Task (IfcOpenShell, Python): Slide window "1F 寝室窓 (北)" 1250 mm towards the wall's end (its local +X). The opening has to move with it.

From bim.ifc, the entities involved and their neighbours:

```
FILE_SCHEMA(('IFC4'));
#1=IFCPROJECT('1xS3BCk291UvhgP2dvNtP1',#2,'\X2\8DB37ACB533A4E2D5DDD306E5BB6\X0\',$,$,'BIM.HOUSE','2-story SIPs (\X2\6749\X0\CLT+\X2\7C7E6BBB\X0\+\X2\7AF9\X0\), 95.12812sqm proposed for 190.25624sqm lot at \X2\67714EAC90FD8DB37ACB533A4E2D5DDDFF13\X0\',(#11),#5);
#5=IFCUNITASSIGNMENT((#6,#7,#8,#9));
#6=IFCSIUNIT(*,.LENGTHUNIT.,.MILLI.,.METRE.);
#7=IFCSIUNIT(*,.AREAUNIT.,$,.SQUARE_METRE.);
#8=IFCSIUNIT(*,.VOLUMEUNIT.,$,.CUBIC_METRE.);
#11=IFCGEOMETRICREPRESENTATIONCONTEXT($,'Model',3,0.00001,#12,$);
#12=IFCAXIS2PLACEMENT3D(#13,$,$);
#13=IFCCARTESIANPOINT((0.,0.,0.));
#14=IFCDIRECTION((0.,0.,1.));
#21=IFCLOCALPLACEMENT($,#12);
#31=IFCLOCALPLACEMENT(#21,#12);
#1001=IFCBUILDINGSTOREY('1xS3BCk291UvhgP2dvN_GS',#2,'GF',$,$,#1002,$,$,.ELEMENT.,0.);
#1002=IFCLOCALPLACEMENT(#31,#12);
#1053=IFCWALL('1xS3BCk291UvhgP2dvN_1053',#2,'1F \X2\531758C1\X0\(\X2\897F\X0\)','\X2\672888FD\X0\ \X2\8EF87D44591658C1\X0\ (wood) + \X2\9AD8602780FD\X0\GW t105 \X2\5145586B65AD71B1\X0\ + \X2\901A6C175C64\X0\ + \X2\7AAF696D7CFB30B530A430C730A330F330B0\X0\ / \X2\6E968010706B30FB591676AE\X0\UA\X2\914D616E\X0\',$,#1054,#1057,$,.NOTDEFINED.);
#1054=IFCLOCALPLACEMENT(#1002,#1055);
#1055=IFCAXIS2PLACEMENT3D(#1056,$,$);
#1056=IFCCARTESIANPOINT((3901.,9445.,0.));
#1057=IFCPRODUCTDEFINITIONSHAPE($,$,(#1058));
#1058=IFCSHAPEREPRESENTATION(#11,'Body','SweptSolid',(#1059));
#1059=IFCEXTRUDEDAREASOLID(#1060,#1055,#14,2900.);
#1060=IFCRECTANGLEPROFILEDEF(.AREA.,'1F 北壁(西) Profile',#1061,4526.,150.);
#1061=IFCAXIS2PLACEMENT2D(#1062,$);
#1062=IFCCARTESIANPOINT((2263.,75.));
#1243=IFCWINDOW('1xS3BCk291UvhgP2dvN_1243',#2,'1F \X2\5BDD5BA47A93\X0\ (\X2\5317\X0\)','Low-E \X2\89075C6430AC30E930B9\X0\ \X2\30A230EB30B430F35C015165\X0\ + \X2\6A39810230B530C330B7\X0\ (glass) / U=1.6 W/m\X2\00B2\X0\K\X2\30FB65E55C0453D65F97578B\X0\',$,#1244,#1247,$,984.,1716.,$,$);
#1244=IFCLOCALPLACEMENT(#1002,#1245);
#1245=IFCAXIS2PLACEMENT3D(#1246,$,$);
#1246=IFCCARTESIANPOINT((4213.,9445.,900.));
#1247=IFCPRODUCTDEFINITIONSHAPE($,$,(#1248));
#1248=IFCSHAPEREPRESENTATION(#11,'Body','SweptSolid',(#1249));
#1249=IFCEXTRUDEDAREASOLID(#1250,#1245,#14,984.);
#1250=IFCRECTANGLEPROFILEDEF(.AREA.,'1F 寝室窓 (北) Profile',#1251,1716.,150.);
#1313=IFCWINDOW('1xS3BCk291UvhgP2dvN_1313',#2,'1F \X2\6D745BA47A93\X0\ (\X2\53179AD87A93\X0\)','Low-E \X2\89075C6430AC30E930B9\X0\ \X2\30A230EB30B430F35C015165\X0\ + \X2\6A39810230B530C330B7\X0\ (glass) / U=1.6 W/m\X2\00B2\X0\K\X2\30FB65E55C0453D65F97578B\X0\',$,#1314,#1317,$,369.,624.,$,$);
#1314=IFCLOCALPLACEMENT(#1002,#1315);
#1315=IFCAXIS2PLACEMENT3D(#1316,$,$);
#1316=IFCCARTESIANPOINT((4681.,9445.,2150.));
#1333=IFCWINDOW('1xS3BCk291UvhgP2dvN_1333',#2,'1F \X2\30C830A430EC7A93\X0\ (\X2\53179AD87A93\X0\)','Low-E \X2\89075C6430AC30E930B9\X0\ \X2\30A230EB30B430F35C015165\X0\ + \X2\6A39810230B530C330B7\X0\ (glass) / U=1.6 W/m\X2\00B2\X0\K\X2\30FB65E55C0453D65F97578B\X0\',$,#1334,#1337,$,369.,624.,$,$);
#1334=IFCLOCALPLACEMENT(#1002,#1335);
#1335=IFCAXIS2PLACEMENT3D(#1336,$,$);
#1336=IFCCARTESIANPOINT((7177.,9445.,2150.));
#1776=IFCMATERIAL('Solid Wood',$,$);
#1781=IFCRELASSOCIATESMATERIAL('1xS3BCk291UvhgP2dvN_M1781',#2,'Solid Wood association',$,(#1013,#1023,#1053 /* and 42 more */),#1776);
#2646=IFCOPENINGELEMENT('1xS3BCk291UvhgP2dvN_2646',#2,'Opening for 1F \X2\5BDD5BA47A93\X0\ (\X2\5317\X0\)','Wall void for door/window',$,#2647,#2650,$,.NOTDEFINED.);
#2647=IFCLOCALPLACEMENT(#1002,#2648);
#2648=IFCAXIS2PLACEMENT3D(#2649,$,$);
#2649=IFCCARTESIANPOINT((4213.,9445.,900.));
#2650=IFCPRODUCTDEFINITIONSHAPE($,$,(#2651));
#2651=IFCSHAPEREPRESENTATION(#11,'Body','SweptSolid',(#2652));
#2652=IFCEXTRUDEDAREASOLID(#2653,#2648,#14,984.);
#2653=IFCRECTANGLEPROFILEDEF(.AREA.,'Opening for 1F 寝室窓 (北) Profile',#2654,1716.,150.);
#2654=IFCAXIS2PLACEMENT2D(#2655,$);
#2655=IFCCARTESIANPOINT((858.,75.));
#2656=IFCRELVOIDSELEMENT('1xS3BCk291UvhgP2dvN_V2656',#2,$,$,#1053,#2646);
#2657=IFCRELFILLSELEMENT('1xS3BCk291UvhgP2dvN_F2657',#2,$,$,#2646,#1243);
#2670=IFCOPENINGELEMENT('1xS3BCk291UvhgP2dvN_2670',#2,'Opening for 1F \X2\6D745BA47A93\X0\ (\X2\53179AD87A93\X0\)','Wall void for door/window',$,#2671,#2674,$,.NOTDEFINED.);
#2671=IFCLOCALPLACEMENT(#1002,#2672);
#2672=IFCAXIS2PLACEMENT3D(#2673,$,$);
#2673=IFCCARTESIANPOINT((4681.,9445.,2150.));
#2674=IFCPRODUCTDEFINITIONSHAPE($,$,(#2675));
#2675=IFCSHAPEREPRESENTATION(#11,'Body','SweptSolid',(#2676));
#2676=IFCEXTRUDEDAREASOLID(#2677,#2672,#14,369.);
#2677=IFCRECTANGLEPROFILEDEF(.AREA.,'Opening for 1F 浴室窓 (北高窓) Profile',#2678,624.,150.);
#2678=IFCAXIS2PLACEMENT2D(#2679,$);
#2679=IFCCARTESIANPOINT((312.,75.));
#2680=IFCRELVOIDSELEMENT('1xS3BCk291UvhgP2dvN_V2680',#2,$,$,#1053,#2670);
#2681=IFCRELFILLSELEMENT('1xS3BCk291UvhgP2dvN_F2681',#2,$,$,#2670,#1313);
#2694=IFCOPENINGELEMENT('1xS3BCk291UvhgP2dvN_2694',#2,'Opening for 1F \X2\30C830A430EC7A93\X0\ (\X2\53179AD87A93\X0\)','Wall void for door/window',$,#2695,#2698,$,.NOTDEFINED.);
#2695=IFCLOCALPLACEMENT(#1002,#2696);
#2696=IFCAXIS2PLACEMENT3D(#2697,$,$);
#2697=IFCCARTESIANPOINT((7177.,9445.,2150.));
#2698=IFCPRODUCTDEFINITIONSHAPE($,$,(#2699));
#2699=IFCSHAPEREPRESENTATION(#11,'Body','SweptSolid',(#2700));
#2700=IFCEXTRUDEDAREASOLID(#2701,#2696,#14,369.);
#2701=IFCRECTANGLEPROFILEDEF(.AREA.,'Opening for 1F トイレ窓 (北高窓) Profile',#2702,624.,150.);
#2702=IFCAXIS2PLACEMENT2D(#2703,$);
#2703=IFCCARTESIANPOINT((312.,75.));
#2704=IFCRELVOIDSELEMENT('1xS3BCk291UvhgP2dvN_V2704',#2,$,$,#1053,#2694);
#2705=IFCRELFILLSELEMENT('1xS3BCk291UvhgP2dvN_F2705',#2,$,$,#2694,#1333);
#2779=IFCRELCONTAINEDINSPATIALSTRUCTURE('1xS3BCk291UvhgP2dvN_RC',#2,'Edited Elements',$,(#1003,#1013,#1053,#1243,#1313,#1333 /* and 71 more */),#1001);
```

```python
import ifcopenshell
import ifcopenshell.api.geometry
import ifcopenshell.util.placement
import ifcopenshell.util.unit

model = ifcopenshell.open("bim.ifc")
unit_scale = ifcopenshell.util.unit.calculate_unit_scale(model)

window = model.by_guid("1xS3BCk291UvhgP2dvN_1243")
opening = window.FillsVoids[0].RelatingOpeningElement
wall = opening.VoidsElements[0].RelatingBuildingElement

wall_matrix = ifcopenshell.util.placement.get_local_placement(wall.ObjectPlacement)
shift = wall_matrix[:3, 0] * 1.25 / unit_scale
before = ifcopenshell.util.placement.get_local_placement(window.ObjectPlacement)[:3, 3].copy()

# The window is not placed relative to its opening, so move both.
for product in (opening, window):
    matrix = ifcopenshell.util.placement.get_local_placement(product.ObjectPlacement)
    matrix[:3, 3] += shift
    ifcopenshell.api.geometry.edit_object_placement(model, product=product, matrix=matrix, is_si=False)

after = ifcopenshell.util.placement.get_local_placement(window.ObjectPlacement)[:3, 3]
print("window moved by", (after - before).round(3) + 0.0)

model.write("bim_updated.ifc")
```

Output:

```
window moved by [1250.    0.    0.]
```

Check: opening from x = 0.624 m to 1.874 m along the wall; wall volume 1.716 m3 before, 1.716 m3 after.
